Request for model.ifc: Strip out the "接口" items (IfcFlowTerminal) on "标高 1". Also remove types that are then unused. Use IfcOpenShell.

First a look at what the model holds.

```python
import ifcopenshell
import ifcopenshell.util.element

model = ifcopenshell.open("model.ifc")
print(model.schema)
storey = next(s for s in model.by_type("IfcBuildingStorey") if s.Name == "标高 1")
terminals = [e for e in ifcopenshell.util.element.get_decomposition(storey) if e.is_a("IfcFlowTerminal")]
seen = {}
for e in terminals:
    element_type = ifcopenshell.util.element.get_type(e)
    name = element_type.Name if element_type not in (None, e) else None
    seen[name] = seen.get(name, 0) + 1
for name, count in sorted(seen.items(), key=str):
    print(count, "x", name)
```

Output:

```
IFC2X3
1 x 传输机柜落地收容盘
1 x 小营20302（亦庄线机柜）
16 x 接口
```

```python
import ifcopenshell
import ifcopenshell.api.root
import ifcopenshell.util.element

model = ifcopenshell.open("model.ifc")

storey = next(s for s in model.by_type("IfcBuildingStorey") if s.Name == "标高 1")
terminals = [e for e in ifcopenshell.util.element.get_decomposition(storey) if e.is_a("IfcFlowTerminal")]
targets = [e for e in terminals if (t := ifcopenshell.util.element.get_type(e)) not in (None, e) and t.Name == "接口"]
types = {ifcopenshell.util.element.get_type(e) for e in targets} - {None, *targets}

for e in targets:
    ifcopenshell.api.root.remove_product(model, product=e)
print(len(targets), "removed")

unused = [t for t in types if not ifcopenshell.util.element.get_types(t)]
for t in unused:
    ifcopenshell.api.root.remove_product(model, product=t)
print(len(unused), "unused types removed")

model.write("model_updated.ifc")
```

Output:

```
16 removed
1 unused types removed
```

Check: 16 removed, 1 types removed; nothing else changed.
